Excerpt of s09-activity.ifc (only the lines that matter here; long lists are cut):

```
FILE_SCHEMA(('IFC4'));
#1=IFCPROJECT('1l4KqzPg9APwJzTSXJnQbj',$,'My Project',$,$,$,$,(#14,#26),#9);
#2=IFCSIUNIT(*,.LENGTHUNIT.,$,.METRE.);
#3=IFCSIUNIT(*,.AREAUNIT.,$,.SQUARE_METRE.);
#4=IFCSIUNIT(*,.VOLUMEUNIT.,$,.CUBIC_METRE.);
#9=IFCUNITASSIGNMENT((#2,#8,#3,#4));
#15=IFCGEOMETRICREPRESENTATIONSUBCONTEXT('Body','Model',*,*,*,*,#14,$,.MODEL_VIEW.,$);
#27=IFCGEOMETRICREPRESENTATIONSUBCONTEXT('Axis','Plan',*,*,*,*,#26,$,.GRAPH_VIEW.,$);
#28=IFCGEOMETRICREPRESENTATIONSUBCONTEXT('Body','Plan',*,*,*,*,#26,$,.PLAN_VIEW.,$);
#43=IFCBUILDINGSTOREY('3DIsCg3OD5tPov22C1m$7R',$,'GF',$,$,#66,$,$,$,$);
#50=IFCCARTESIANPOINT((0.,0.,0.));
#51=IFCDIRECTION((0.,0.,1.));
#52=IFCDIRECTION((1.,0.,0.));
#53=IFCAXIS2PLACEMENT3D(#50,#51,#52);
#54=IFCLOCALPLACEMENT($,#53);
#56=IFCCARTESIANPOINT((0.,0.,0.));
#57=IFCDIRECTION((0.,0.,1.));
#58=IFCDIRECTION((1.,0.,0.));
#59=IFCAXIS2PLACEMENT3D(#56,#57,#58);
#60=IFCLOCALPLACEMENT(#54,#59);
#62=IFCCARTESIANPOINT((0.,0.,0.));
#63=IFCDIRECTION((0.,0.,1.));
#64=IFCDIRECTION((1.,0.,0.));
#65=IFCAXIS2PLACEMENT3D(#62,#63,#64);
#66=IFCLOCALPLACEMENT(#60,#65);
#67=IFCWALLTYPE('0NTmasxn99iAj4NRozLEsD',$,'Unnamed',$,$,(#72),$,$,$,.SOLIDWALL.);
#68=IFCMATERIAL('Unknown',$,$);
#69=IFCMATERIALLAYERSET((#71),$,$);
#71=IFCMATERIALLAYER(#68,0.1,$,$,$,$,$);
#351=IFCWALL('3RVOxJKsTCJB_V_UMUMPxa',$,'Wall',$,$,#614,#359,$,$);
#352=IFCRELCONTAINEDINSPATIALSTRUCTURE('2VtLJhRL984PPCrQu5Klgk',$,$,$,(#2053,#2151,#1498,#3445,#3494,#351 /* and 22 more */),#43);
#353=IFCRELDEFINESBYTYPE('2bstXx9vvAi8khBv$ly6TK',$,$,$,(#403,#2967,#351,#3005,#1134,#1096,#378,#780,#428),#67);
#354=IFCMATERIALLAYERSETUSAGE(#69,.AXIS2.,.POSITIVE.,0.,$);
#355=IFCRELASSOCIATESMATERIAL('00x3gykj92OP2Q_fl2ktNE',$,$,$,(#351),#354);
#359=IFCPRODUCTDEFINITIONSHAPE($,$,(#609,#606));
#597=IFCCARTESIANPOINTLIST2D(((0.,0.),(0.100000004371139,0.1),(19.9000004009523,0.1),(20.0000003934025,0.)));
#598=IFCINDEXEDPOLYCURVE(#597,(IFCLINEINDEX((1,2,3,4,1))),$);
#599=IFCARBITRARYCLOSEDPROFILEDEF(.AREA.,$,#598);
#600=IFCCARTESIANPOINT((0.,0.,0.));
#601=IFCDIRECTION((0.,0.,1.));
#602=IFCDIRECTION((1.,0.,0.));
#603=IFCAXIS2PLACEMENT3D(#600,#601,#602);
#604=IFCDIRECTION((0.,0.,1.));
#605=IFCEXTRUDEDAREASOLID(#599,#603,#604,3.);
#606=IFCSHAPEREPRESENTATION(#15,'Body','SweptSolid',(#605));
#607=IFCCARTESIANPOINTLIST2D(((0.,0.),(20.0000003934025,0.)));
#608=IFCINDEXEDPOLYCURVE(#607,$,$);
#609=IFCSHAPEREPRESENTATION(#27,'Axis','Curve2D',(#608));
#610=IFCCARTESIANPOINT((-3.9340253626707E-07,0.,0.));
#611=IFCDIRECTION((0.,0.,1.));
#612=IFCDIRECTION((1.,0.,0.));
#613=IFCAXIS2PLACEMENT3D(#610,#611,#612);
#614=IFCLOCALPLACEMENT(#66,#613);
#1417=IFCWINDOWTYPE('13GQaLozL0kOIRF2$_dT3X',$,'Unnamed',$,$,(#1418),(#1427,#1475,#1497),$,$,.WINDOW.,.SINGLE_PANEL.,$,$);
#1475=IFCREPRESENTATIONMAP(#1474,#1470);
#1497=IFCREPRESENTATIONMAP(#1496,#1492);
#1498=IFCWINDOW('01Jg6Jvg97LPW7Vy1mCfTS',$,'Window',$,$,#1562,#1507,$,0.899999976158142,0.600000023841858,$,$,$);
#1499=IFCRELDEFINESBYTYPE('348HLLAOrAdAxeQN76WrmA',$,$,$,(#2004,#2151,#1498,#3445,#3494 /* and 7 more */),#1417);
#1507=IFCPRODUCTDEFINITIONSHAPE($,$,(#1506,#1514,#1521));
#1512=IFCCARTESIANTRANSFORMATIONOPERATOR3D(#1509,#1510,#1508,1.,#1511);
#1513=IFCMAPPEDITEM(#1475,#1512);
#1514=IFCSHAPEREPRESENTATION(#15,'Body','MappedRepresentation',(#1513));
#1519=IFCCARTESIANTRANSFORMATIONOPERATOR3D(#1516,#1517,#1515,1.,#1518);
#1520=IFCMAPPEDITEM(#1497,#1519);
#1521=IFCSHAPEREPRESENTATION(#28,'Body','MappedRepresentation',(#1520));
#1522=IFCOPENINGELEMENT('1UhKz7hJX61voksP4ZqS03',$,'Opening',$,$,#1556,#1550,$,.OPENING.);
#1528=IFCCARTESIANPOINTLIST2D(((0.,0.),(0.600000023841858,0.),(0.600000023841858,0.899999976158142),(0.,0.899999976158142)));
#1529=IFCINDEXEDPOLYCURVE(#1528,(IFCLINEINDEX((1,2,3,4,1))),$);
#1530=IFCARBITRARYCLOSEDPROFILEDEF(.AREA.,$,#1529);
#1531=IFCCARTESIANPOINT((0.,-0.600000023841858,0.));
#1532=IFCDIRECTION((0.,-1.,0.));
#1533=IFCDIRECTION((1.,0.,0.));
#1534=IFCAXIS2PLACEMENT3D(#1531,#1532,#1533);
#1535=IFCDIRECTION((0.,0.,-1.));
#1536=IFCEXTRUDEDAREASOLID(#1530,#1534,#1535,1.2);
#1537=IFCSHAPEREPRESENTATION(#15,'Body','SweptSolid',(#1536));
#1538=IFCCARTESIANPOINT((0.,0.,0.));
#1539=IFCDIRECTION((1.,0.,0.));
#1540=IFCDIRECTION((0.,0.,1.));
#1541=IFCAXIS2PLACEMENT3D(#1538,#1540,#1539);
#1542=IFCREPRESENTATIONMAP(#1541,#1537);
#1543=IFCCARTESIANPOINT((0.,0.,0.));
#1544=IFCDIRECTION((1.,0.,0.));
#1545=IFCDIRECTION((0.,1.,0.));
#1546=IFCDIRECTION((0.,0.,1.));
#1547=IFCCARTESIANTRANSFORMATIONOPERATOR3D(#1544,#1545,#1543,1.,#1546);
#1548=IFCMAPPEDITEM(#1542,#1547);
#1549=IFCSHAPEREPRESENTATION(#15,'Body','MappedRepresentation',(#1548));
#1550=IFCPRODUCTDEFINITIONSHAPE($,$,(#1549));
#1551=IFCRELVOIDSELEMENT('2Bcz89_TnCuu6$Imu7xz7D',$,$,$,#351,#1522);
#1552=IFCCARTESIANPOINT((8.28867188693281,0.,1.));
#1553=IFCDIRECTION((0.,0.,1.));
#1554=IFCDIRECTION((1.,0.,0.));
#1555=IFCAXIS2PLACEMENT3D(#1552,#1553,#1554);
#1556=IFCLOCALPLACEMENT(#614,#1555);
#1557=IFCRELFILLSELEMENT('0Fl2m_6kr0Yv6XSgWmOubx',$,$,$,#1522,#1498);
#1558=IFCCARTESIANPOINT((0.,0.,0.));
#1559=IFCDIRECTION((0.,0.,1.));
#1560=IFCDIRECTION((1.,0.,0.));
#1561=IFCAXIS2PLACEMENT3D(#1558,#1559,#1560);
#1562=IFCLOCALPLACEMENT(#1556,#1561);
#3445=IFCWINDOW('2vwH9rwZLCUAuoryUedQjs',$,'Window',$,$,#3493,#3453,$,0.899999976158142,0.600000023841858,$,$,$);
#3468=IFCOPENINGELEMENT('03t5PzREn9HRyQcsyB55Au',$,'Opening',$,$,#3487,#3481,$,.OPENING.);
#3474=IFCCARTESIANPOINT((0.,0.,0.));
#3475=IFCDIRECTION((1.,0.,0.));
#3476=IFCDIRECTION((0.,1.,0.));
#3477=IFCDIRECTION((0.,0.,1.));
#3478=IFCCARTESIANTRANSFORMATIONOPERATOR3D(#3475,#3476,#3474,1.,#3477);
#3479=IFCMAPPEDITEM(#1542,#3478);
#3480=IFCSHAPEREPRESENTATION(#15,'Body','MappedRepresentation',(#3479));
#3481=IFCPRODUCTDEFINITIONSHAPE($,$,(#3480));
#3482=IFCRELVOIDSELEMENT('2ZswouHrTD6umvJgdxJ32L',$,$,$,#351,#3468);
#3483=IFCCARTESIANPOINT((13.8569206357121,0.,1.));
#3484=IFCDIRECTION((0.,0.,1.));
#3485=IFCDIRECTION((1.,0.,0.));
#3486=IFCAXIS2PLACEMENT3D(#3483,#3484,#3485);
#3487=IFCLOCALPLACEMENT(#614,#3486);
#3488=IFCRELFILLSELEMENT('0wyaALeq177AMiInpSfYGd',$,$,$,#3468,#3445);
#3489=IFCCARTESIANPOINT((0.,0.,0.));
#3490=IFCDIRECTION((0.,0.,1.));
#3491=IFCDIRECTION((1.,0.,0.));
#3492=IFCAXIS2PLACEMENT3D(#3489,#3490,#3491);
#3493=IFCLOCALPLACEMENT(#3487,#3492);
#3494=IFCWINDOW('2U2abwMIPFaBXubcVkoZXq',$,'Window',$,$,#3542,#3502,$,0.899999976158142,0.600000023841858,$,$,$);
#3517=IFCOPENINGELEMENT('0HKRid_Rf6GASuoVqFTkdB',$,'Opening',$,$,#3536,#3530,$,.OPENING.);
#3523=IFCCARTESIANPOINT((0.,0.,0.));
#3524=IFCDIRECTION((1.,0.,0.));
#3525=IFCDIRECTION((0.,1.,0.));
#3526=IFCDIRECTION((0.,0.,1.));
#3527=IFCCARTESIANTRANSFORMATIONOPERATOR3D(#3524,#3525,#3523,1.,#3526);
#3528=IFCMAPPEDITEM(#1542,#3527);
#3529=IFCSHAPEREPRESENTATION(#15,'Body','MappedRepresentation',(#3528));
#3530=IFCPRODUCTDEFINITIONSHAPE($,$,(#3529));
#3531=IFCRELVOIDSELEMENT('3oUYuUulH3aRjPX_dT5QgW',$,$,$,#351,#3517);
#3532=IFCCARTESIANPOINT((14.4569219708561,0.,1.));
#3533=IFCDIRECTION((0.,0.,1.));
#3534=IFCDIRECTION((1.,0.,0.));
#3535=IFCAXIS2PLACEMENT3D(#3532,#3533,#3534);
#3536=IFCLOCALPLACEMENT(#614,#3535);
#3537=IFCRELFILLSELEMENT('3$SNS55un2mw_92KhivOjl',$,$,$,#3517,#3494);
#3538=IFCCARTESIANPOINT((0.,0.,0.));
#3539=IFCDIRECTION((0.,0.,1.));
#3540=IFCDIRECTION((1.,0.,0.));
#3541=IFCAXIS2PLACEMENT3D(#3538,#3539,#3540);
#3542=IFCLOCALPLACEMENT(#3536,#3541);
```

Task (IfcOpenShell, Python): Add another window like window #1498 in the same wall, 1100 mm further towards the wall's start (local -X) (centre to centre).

```python
import ifcopenshell
import ifcopenshell.api.feature
import ifcopenshell.api.geometry
import ifcopenshell.api.root
import ifcopenshell.geom
import ifcopenshell.util.element
import ifcopenshell.util.placement
import ifcopenshell.util.shape
import ifcopenshell.util.unit

model = ifcopenshell.open("s09-activity.ifc")
unit_scale = ifcopenshell.util.unit.calculate_unit_scale(model)
settings = ifcopenshell.geom.settings()


def volume(element):
    """Net volume in cubic metres, openings subtracted."""
    shape = ifcopenshell.geom.create_shape(settings, element)
    return ifcopenshell.util.shape.get_volume(shape.geometry)


window = model.by_guid("01Jg6Jvg97LPW7Vy1mCfTS")
opening = window.FillsVoids[0].RelatingOpeningElement
wall = opening.VoidsElements[0].RelatingBuildingElement
before = volume(wall)
shift = ifcopenshell.util.placement.get_local_placement(wall.ObjectPlacement)[:3, 0] * -1.1 / unit_scale

# copy_class copies the void relationship, type, container and properties, but no geometry.
new_opening = ifcopenshell.api.root.copy_class(model, product=opening)
new_opening.Representation = ifcopenshell.util.element.copy_deep(
    model, opening.Representation, exclude=["IfcGeometricRepresentationContext", "IfcRepresentationMap"]
)
new_window = ifcopenshell.api.root.copy_class(model, product=window)
new_window.Representation = ifcopenshell.util.element.copy_deep(
    model, window.Representation, exclude=["IfcGeometricRepresentationContext", "IfcRepresentationMap"]
)
ifcopenshell.api.feature.add_filling(model, opening=new_opening, element=new_window)

for old, new in ((opening, new_opening), (window, new_window)):
    matrix = ifcopenshell.util.placement.get_local_placement(old.ObjectPlacement)
    matrix[:3, 3] += shift
    ifcopenshell.api.geometry.edit_object_placement(model, product=new, matrix=matrix, is_si=False)

after = volume(wall)

print(f"wall volume {before:.3f} -> {after:.3f} m3")

model.write("s09-activity-out.ifc")
```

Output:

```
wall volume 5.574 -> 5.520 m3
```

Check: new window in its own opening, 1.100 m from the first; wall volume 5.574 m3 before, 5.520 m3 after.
